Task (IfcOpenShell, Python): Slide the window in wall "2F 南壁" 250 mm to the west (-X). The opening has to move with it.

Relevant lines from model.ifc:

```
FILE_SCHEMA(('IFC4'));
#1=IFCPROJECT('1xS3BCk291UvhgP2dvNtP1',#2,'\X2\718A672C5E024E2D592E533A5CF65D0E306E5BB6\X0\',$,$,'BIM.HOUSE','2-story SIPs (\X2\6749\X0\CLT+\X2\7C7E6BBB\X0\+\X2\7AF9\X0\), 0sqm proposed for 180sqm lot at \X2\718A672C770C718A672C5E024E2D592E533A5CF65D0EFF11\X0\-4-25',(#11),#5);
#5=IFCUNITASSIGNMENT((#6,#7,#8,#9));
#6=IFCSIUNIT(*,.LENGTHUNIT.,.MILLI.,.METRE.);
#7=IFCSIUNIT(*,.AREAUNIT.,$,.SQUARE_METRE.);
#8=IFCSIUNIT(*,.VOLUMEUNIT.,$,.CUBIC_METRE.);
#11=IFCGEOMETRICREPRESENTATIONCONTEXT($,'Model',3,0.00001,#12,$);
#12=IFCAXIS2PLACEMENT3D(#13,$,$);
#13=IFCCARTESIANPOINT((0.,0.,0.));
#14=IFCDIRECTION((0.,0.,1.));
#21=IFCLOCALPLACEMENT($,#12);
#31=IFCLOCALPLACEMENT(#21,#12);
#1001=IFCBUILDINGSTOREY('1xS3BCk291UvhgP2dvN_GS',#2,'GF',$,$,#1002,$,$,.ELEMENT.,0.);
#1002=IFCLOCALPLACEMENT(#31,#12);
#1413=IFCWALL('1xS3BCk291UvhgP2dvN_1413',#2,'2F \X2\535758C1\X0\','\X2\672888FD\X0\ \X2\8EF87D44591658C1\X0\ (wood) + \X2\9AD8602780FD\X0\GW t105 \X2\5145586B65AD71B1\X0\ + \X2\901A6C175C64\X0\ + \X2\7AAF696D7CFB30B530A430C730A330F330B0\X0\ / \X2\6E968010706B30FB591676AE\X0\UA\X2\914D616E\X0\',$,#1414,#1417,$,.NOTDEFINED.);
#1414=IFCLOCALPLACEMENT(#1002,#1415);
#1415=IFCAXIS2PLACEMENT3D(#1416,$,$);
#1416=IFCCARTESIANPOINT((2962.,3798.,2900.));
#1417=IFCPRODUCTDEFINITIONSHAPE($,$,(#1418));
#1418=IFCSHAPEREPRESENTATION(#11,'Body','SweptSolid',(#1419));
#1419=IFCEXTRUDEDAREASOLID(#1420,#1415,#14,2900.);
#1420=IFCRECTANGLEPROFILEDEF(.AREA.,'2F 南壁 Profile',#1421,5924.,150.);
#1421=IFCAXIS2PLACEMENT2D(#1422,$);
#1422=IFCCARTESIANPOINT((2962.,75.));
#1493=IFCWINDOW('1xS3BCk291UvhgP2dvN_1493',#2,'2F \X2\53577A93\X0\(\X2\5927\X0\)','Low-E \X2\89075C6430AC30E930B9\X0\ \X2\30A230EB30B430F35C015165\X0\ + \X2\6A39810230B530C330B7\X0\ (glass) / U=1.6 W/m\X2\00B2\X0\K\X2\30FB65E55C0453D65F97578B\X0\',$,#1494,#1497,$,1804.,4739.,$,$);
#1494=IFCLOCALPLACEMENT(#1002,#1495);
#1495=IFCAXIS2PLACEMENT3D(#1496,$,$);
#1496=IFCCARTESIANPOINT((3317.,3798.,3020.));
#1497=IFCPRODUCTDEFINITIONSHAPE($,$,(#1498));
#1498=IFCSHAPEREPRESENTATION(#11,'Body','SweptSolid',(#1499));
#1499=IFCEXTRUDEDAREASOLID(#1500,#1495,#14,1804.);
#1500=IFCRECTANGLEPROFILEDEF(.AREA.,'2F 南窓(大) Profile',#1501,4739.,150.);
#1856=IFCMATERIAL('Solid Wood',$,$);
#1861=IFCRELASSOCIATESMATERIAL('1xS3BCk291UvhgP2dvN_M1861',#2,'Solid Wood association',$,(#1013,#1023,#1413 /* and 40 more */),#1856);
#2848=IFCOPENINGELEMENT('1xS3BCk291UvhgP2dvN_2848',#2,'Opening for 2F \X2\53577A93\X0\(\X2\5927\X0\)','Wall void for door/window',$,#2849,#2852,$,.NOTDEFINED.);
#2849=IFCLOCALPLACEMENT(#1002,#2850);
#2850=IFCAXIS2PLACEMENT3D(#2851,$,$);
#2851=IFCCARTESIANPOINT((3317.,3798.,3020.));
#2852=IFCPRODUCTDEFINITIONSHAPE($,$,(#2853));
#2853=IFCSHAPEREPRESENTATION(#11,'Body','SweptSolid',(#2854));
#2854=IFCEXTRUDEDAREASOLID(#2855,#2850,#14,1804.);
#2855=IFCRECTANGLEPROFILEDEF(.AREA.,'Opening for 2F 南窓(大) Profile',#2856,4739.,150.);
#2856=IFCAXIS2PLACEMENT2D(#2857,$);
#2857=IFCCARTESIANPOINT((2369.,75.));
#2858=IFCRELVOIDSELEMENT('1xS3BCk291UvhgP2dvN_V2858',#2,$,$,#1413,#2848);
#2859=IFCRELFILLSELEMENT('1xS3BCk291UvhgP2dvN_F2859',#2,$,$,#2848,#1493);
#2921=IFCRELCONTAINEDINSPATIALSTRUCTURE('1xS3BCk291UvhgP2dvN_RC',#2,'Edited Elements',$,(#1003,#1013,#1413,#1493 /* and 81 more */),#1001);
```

```python
import ifcopenshell
import ifcopenshell.api.geometry
import ifcopenshell.util.placement
import ifcopenshell.util.unit

model = ifcopenshell.open("model.ifc")
unit_scale = ifcopenshell.util.unit.calculate_unit_scale(model)

window = model.by_guid("1xS3BCk291UvhgP2dvN_1493")
opening = window.FillsVoids[0].RelatingOpeningElement
wall = opening.VoidsElements[0].RelatingBuildingElement

wall_matrix = ifcopenshell.util.placement.get_local_placement(wall.ObjectPlacement)
shift = wall_matrix[:3, 0] * -0.25 / unit_scale
before = ifcopenshell.util.placement.get_local_placement(window.ObjectPlacement)[:3, 3].copy()

# The window is not placed relative to its opening, so move both.
for product in (opening, window):
    matrix = ifcopenshell.util.placement.get_local_placement(product.ObjectPlacement)
    matrix[:3, 3] += shift
    ifcopenshell.api.geometry.edit_object_placement(model, product=product, matrix=matrix, is_si=False)

after = ifcopenshell.util.placement.get_local_placement(window.ObjectPlacement)[:3, 3]
print("window moved by", (after - before).round(3) + 0.0)

model.write("model-out.ifc")
```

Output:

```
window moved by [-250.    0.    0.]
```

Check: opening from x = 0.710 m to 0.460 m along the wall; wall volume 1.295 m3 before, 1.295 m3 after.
